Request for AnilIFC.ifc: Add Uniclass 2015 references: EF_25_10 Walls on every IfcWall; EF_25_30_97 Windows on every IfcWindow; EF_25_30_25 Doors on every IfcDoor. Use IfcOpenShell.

First a look at what the model holds.

```python
import ifcopenshell

model = ifcopenshell.open("AnilIFC.ifc")
print(model.schema)
print("classifications:", [c.Name for c in model.by_type("IfcClassification")])
for ifc_class in ("IfcDoor", "IfcRoof", "IfcStair", "IfcWall", "IfcWindow"):
    print(ifc_class, len(model.by_type(ifc_class)))
```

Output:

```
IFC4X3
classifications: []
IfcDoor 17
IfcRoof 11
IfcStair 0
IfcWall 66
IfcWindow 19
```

```python
import ifcopenshell
import ifcopenshell.api.classification

model = ifcopenshell.open("AnilIFC.ifc")

system = ifcopenshell.api.classification.add_classification(model, classification="Uniclass 2015")

codes = {
    "IfcWall": ("EF_25_10", "Walls"),
    "IfcWindow": ("EF_25_30_97", "Windows"),
    "IfcDoor": ("EF_25_30_25", "Doors"),
}
for ifc_class, (code, name) in codes.items():
    products = model.by_type(ifc_class)
    ifcopenshell.api.classification.add_reference(
        model, products=products, classification=system, identification=code, name=name
    )
    print(code, len(products))

model.write("AnilIFC_rev.ifc")
```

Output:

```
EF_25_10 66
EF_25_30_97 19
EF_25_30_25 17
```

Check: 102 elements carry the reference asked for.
